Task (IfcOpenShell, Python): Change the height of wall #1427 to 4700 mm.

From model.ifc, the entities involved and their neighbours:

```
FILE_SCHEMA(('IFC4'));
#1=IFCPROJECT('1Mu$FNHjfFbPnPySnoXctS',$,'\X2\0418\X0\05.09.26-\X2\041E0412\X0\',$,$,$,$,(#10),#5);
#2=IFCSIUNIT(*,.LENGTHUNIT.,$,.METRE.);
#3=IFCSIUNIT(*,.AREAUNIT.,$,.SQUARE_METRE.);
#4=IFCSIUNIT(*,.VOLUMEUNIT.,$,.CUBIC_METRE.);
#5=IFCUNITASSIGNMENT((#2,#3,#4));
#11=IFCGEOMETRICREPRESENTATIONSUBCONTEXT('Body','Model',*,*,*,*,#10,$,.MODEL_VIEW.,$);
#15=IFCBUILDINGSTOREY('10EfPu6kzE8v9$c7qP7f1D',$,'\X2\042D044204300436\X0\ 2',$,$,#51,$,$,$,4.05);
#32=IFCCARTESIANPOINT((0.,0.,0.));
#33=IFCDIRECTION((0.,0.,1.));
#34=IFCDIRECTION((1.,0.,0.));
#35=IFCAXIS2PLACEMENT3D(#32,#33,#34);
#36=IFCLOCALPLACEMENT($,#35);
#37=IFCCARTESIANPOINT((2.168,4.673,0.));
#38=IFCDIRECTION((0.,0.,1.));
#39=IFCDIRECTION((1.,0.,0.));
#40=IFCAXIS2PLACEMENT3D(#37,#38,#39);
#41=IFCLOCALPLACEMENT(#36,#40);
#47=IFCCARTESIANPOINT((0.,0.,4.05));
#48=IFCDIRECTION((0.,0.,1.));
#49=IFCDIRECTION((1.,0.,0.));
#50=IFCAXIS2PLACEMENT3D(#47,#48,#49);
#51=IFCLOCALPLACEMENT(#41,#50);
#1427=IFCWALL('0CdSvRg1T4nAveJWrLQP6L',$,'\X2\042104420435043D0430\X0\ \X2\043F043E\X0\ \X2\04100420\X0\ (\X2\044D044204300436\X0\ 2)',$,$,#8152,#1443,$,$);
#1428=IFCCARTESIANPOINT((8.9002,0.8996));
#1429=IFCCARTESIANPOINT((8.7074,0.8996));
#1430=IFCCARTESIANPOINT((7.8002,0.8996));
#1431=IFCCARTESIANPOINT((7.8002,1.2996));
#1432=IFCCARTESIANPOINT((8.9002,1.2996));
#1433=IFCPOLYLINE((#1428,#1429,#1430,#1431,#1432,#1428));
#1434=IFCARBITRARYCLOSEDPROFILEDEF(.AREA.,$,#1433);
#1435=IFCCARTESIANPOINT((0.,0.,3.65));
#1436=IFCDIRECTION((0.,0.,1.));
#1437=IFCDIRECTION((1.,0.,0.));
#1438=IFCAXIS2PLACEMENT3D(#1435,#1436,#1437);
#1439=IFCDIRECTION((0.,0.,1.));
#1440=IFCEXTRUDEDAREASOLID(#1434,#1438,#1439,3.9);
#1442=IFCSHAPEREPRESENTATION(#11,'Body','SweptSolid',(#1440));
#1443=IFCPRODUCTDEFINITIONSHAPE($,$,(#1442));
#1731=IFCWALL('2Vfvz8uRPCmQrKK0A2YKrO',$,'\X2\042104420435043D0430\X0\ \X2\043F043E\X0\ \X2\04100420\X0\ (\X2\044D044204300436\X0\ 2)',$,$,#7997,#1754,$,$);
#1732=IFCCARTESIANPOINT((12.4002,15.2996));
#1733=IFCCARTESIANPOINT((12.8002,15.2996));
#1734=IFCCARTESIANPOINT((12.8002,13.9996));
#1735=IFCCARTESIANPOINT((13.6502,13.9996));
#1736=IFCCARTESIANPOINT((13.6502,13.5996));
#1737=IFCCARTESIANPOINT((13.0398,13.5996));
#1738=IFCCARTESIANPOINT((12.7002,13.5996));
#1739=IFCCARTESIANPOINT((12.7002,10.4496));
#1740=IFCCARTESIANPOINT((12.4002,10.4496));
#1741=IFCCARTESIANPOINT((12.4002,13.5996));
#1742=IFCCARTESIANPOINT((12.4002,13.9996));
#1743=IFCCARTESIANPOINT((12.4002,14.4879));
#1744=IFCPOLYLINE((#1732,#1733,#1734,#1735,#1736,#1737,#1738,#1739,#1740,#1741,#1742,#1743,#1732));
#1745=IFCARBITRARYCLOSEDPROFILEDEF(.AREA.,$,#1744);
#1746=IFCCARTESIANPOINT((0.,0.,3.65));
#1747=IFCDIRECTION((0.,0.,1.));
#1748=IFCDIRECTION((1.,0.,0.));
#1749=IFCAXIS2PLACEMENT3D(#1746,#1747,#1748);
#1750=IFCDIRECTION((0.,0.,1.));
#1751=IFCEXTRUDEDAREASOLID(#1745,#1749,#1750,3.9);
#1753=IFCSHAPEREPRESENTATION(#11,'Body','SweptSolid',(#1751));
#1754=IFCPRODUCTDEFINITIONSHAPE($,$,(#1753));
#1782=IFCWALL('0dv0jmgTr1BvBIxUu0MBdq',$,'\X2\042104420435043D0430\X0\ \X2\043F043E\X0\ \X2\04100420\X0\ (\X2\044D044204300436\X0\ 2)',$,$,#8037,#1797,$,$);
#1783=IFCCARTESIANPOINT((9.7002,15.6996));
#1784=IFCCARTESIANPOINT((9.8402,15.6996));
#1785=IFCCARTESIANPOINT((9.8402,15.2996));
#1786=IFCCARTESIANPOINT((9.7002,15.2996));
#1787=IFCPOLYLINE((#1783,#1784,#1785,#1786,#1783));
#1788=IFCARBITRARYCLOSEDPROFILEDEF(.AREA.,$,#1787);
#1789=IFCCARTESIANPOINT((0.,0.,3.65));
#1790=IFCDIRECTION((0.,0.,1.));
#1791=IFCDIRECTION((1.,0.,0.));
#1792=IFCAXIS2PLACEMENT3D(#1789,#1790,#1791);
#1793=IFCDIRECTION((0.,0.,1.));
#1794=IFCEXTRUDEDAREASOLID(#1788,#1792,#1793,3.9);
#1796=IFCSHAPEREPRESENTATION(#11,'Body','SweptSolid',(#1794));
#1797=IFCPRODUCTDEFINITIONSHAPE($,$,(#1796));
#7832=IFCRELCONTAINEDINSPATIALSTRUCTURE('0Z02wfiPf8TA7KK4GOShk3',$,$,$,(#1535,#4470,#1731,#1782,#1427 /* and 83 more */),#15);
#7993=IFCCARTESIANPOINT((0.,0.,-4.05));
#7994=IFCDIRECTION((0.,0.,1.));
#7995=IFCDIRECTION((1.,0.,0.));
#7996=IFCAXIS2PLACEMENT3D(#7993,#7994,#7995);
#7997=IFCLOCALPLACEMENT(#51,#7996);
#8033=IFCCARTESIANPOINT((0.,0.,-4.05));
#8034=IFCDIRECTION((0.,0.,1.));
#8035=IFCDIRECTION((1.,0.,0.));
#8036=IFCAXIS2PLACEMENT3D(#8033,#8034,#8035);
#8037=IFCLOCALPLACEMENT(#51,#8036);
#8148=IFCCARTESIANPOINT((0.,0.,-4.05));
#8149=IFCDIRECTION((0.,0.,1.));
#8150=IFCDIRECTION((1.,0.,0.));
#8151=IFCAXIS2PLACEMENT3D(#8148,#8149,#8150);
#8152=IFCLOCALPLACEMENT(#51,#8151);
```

```python
import ifcopenshell
import ifcopenshell.geom
import ifcopenshell.util.representation
import ifcopenshell.util.shape
import ifcopenshell.util.unit

model = ifcopenshell.open("model.ifc")
unit_scale = ifcopenshell.util.unit.calculate_unit_scale(model)
settings = ifcopenshell.geom.settings()


def volume(element):
    """Net volume in cubic metres, openings subtracted."""
    shape = ifcopenshell.geom.create_shape(settings, element)
    return ifcopenshell.util.shape.get_volume(shape.geometry)


wall = model.by_guid("0CdSvRg1T4nAveJWrLQP6L")
before = volume(wall)

body = ifcopenshell.util.representation.get_representation(wall, "Model", "Body")
solid = body.Items[0]
old_height = solid.Depth
solid.Depth = 4.7 / unit_scale
after = volume(wall)

print(f"height {old_height:g} -> {solid.Depth:g}, volume {before:.3f} -> {after:.3f} m3")

model.write("model_updated.ifc")
```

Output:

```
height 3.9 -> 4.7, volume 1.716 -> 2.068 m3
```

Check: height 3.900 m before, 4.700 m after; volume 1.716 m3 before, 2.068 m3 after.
